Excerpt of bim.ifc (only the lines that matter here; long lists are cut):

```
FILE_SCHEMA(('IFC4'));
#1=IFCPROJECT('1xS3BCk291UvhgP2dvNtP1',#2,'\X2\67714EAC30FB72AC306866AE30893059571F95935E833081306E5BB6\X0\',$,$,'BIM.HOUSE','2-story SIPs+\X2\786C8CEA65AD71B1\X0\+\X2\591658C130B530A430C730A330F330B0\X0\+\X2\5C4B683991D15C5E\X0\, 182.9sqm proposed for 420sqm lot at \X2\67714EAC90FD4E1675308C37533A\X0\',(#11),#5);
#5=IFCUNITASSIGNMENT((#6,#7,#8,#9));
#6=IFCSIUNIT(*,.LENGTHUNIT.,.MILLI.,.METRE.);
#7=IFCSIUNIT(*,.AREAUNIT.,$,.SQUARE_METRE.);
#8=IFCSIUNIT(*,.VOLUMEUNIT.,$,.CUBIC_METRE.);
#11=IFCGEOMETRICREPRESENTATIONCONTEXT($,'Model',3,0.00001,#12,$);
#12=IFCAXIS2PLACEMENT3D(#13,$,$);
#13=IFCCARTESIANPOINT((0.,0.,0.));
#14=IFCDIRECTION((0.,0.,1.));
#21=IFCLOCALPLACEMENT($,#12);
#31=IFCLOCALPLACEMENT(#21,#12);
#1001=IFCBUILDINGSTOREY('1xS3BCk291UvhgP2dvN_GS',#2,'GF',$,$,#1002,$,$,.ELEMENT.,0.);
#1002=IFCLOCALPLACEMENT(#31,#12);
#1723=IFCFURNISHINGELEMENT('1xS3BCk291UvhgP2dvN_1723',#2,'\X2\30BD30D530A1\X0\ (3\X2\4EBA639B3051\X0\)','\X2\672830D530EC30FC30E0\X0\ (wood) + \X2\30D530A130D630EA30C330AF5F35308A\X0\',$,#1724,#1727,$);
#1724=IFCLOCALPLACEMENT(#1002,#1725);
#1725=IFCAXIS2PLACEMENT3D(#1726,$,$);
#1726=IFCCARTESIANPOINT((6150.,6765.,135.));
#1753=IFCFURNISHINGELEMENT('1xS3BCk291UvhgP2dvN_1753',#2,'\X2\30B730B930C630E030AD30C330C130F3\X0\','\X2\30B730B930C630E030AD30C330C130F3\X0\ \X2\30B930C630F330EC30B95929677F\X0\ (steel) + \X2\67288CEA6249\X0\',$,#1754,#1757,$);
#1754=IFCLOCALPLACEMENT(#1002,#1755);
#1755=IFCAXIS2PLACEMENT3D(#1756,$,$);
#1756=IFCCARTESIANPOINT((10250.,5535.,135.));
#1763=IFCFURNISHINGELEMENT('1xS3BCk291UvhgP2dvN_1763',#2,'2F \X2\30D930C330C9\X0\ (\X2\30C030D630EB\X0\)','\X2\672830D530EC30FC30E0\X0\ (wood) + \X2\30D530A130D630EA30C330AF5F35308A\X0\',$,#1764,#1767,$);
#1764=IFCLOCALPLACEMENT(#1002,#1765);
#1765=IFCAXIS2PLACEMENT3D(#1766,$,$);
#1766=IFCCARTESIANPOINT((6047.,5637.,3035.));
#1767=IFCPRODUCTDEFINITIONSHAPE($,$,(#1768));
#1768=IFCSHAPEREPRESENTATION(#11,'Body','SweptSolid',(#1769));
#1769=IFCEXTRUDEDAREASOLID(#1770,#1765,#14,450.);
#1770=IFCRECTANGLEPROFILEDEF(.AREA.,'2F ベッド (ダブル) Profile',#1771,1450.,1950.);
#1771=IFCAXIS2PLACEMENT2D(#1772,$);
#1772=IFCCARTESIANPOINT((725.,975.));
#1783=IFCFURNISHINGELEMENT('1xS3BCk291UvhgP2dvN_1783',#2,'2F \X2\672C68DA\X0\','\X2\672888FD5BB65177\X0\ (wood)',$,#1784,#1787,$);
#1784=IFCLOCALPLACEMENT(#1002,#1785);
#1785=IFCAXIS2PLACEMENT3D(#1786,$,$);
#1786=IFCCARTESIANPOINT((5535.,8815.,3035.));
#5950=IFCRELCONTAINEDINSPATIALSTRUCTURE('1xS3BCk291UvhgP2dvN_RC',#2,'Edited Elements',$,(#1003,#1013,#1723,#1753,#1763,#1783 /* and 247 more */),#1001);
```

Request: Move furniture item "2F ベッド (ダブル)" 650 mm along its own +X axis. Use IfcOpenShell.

```python
import ifcopenshell
import ifcopenshell.api.geometry
import ifcopenshell.util.placement

model = ifcopenshell.open("bim.ifc")

item = model.by_guid("1xS3BCk291UvhgP2dvN_1763")
matrix = ifcopenshell.util.placement.get_local_placement(item.ObjectPlacement)
matrix[:3, 3] += matrix[:3, 0] * 650.0
ifcopenshell.api.geometry.edit_object_placement(model, product=item, matrix=matrix, is_si=False)

print(ifcopenshell.util.placement.get_local_placement(item.ObjectPlacement).round(3) + 0.0)

model.write("bim-out.ifc")
```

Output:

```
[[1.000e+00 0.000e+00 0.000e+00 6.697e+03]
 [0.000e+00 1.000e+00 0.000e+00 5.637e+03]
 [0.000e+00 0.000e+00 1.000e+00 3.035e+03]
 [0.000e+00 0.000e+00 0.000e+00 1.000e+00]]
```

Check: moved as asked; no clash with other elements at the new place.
